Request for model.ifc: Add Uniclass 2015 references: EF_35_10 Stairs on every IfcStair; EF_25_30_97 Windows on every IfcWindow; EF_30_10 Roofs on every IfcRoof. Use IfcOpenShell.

First a look at what the model holds.

```python
import ifcopenshell

model = ifcopenshell.open("model.ifc")
print(model.schema)
print("classifications:", [c.Name for c in model.by_type("IfcClassification")])
for ifc_class in ("IfcDoor", "IfcRoof", "IfcStair", "IfcWall", "IfcWindow"):
    print(ifc_class, len(model.by_type(ifc_class)))
```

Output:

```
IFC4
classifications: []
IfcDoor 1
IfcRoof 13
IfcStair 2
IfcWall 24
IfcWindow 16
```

```python
import ifcopenshell
import ifcopenshell.api.classification

model = ifcopenshell.open("model.ifc")

system = ifcopenshell.api.classification.add_classification(model, classification="Uniclass 2015")

codes = {
    "IfcStair": ("EF_35_10", "Stairs"),
    "IfcWindow": ("EF_25_30_97", "Windows"),
    "IfcRoof": ("EF_30_10", "Roofs"),
}
for ifc_class, (code, name) in codes.items():
    products = model.by_type(ifc_class)
    ifcopenshell.api.classification.add_reference(
        model, products=products, classification=system, identification=code, name=name
    )
    print(code, len(products))

model.write("model_updated.ifc")
```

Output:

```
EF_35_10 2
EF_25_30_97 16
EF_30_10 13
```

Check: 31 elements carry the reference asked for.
